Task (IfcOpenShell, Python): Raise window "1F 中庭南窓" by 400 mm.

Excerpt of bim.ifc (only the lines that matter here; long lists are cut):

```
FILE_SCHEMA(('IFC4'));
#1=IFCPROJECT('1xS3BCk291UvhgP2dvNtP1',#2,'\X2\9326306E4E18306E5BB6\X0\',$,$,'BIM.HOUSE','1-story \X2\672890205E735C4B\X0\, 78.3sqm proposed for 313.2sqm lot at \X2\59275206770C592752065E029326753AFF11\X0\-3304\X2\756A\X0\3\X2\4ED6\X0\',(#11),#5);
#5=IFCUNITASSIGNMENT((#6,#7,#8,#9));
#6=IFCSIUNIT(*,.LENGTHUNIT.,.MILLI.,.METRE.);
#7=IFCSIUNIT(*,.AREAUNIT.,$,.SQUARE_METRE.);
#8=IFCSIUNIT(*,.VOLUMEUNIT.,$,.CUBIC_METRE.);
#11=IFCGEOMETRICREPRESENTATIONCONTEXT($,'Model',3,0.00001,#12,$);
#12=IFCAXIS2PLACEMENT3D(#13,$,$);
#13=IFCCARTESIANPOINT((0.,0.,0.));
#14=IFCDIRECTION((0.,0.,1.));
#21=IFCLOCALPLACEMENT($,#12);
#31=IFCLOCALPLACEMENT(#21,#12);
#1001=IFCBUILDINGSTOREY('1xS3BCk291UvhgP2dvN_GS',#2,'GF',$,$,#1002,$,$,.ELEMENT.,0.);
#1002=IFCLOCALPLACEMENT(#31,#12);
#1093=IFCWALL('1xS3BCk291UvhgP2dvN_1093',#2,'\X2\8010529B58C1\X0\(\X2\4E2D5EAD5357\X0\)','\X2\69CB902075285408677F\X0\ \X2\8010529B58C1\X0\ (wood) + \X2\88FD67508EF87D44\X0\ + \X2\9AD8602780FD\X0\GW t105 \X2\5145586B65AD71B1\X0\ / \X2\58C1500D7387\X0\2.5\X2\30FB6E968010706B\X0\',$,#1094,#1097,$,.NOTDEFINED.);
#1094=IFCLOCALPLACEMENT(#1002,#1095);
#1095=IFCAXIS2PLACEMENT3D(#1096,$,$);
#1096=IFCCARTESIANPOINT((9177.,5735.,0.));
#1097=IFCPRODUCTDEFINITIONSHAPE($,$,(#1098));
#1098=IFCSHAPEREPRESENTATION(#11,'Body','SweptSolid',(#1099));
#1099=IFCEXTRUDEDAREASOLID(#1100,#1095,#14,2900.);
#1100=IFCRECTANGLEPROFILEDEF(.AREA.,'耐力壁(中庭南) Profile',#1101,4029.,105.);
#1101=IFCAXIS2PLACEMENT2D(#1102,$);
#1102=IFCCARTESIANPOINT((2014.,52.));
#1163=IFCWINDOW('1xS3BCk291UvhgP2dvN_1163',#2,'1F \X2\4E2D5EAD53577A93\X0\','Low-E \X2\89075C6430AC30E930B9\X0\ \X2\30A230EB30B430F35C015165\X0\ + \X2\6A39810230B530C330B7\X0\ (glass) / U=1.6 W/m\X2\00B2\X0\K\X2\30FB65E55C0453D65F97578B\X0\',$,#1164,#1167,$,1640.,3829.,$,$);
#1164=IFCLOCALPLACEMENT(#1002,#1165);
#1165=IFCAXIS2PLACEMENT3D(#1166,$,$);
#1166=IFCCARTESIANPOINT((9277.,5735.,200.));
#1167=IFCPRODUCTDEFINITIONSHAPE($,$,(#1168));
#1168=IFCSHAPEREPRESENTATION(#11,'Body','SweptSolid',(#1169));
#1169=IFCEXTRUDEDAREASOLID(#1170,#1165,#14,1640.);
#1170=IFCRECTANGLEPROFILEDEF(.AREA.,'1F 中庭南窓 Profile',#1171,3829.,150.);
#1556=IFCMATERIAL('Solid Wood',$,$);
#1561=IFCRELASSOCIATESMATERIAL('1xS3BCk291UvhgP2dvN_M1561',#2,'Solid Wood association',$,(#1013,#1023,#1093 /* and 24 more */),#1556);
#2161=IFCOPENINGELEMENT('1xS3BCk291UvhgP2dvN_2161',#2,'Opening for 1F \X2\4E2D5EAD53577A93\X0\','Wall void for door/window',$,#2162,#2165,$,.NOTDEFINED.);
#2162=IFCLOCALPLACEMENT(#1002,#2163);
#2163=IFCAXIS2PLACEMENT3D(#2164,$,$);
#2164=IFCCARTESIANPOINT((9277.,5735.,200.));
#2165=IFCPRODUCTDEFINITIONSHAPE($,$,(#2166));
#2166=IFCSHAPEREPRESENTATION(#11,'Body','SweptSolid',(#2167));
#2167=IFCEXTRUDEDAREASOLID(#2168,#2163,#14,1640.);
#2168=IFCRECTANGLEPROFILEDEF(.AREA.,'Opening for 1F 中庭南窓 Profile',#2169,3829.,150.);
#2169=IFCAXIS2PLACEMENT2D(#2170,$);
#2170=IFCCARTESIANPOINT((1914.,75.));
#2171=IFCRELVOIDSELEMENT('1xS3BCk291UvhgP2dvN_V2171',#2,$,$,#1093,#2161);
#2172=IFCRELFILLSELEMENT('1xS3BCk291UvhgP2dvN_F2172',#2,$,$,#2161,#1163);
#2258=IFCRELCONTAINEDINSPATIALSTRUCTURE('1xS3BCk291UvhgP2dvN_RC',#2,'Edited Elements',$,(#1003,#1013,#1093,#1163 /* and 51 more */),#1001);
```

```python
import numpy as np
import ifcopenshell
import ifcopenshell.api.geometry
import ifcopenshell.util.placement
import ifcopenshell.util.unit

model = ifcopenshell.open("bim.ifc")
unit_scale = ifcopenshell.util.unit.calculate_unit_scale(model)

window = model.by_id(1163)
opening = window.FillsVoids[0].RelatingOpeningElement
dz = 400.0

shift = np.array([0.0, 0.0, dz])
# The window is not placed relative to its opening, so move both.
for product in (opening, window):
    matrix = ifcopenshell.util.placement.get_local_placement(product.ObjectPlacement)
    matrix[:3, 3] += shift
    ifcopenshell.api.geometry.edit_object_placement(model, product=product, matrix=matrix, is_si=False)

print(f"moved by {dz * unit_scale:+.3f} m")

model.write("bim_v2.ifc")
```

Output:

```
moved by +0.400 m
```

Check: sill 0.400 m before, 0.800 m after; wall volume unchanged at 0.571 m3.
